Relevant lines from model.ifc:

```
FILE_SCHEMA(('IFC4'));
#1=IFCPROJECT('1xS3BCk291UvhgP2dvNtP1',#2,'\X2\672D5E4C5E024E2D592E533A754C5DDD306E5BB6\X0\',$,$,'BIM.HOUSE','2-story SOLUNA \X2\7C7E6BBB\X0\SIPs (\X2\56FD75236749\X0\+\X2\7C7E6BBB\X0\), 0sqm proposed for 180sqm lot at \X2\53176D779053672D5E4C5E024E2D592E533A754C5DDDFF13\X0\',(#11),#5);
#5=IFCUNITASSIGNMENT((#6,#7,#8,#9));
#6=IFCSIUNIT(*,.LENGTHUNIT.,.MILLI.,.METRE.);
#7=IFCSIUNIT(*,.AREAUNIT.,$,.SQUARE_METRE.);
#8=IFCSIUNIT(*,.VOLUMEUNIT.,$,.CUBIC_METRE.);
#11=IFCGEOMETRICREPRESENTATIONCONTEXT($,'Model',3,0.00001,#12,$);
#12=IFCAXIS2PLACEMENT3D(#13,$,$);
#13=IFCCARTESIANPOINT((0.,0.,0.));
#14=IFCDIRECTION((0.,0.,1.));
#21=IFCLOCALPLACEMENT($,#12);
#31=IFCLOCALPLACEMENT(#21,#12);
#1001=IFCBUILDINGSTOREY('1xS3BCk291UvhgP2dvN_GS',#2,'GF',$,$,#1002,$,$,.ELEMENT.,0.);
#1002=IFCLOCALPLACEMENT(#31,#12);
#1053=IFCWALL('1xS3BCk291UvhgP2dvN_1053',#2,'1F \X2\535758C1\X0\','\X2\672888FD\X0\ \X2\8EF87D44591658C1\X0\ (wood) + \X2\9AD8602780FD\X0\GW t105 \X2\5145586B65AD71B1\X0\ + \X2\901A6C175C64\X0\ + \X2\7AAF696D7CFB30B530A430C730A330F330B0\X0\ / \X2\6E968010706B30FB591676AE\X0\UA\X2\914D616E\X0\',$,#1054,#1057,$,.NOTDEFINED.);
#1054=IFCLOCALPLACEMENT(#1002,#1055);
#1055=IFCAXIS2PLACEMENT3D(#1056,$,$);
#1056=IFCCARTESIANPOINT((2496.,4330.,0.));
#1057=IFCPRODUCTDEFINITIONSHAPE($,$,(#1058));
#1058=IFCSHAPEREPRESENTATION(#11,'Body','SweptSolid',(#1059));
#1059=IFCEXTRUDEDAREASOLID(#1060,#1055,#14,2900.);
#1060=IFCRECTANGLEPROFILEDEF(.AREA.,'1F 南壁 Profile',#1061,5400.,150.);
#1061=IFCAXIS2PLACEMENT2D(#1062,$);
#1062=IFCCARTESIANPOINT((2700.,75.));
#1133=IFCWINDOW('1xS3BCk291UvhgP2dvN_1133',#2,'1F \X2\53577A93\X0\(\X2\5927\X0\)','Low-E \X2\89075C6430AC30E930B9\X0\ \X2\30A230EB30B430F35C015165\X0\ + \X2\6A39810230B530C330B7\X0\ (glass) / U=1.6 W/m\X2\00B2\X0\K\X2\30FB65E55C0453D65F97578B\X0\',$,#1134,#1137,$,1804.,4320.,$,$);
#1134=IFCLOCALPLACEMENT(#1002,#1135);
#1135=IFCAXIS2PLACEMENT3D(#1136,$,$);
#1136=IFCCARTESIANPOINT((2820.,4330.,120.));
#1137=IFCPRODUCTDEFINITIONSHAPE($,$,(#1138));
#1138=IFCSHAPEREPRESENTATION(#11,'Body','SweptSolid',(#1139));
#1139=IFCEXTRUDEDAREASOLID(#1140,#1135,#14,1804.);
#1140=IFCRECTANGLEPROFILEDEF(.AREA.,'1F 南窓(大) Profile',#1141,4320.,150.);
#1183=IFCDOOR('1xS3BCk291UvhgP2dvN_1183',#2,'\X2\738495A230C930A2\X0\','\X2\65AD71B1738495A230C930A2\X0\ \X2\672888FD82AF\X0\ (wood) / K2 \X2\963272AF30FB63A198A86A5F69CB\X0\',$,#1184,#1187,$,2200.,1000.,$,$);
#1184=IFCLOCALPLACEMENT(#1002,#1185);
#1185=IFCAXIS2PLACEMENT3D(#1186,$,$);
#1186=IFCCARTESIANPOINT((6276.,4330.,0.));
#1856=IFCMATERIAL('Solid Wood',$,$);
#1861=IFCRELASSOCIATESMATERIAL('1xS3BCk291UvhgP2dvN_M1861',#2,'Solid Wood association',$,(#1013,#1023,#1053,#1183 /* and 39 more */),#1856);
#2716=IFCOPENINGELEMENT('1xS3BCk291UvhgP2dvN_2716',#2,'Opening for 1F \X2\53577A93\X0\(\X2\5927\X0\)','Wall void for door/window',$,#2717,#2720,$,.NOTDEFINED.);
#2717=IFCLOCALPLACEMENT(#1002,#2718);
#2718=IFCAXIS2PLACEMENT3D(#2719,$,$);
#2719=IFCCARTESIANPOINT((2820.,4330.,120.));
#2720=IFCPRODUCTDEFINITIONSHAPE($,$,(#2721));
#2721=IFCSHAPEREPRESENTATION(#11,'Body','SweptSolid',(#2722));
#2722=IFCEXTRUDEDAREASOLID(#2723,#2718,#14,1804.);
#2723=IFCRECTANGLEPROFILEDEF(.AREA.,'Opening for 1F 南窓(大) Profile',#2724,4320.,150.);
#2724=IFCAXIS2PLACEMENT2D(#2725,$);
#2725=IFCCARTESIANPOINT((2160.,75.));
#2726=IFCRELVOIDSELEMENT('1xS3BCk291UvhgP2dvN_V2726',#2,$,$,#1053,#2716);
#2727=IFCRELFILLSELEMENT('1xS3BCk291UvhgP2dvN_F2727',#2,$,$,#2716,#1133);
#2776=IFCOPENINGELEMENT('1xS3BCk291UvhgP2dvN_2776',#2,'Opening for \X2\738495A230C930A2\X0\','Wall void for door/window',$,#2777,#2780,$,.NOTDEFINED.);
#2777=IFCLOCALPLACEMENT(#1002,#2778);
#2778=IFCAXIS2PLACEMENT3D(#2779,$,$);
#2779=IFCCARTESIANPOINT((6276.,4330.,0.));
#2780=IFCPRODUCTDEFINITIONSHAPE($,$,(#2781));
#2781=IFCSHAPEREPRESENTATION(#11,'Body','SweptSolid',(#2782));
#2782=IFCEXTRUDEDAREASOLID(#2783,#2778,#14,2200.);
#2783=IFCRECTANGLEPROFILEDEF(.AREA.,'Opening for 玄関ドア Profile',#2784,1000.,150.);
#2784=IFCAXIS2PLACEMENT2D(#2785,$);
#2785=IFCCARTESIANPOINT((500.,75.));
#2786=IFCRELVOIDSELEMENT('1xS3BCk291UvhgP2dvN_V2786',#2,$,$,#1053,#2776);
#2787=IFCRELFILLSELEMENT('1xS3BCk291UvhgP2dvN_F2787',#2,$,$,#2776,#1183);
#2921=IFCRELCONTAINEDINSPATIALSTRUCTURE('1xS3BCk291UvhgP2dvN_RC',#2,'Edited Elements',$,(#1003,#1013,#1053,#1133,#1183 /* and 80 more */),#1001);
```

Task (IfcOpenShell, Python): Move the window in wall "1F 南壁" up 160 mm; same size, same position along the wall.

```python
import numpy as np
import ifcopenshell
import ifcopenshell.api.geometry
import ifcopenshell.util.placement
import ifcopenshell.util.unit

model = ifcopenshell.open("model.ifc")
unit_scale = ifcopenshell.util.unit.calculate_unit_scale(model)

window = model.by_guid("1xS3BCk291UvhgP2dvN_1133")
opening = window.FillsVoids[0].RelatingOpeningElement
dz = 160.0

shift = np.array([0.0, 0.0, dz])
# The window is not placed relative to its opening, so move both.
for product in (opening, window):
    matrix = ifcopenshell.util.placement.get_local_placement(product.ObjectPlacement)
    matrix[:3, 3] += shift
    ifcopenshell.api.geometry.edit_object_placement(model, product=product, matrix=matrix, is_si=False)

print(f"moved by {dz * unit_scale:+.3f} m")

model.write("model_edited.ifc")
```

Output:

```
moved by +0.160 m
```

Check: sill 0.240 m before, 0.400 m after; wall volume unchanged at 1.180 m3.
